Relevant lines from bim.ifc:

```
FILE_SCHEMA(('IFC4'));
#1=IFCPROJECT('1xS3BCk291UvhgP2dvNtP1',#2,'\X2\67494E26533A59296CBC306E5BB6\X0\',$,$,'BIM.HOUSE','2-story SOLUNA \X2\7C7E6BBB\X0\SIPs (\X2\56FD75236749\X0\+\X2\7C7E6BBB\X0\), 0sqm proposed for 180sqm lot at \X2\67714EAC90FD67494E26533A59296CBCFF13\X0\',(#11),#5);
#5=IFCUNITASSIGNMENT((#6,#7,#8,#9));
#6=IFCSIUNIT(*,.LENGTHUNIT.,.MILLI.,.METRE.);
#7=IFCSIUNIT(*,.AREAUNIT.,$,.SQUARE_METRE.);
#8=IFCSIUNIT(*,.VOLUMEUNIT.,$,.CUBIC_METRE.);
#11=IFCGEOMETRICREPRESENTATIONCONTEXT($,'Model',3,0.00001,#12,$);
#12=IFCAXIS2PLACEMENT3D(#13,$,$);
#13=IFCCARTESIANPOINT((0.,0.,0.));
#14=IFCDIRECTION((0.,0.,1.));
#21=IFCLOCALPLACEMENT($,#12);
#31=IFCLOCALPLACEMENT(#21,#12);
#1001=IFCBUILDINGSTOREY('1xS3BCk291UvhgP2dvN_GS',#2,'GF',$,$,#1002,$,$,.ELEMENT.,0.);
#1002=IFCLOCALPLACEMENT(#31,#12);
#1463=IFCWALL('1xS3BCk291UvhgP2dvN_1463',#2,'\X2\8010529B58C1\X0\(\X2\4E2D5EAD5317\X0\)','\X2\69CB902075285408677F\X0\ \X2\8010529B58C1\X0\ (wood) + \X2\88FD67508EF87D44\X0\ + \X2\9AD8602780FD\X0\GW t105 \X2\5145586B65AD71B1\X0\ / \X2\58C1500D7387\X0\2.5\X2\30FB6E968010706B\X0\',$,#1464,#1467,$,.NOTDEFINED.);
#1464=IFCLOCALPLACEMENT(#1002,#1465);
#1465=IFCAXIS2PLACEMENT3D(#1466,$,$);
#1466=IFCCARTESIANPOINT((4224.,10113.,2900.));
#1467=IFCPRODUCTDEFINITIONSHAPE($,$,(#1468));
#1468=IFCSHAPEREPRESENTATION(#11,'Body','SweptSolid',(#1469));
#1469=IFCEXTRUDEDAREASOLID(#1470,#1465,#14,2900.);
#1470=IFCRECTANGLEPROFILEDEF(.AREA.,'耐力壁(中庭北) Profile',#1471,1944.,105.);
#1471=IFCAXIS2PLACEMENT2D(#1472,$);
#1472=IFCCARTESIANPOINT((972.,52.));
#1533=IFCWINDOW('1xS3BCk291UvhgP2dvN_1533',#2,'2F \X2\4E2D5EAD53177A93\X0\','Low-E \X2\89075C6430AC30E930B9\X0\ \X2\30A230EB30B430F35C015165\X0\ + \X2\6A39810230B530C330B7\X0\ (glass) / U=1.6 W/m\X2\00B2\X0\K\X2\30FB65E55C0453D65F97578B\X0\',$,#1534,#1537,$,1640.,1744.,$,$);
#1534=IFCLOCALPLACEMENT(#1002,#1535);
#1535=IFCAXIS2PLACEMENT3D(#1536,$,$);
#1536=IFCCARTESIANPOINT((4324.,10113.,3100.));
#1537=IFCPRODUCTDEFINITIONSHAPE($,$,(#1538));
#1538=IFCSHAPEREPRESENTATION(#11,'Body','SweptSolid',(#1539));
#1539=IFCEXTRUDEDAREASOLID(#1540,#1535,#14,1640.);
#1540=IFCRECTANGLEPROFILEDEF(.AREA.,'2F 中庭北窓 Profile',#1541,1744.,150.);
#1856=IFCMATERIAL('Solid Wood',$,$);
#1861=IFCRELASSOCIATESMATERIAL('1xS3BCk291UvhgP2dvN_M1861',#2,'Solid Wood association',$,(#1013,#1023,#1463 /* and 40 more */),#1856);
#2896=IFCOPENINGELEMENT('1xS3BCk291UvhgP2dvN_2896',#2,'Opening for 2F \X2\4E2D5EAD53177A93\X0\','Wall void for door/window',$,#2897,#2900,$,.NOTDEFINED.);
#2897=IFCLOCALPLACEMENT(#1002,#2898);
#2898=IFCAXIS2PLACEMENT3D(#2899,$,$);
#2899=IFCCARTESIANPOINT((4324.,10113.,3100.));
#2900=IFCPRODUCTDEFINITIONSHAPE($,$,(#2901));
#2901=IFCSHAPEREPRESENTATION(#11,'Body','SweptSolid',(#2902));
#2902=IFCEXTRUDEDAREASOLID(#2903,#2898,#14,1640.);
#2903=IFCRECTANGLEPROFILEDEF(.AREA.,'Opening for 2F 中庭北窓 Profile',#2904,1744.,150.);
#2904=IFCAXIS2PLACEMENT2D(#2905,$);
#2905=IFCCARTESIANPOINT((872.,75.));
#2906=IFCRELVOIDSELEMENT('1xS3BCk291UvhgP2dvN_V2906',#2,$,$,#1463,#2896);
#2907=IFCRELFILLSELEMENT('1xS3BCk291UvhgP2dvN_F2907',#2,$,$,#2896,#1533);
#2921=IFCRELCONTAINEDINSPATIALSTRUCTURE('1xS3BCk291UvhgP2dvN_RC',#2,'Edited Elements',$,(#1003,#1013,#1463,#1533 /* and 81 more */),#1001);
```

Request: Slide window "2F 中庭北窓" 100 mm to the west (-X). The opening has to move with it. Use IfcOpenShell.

```python
import ifcopenshell
import ifcopenshell.api.geometry
import ifcopenshell.util.placement

model = ifcopenshell.open("bim.ifc")

window = model.by_guid("1xS3BCk291UvhgP2dvN_1533")
opening = window.FillsVoids[0].RelatingOpeningElement
wall = opening.VoidsElements[0].RelatingBuildingElement

wall_matrix = ifcopenshell.util.placement.get_local_placement(wall.ObjectPlacement)
shift = wall_matrix[:3, 0] * -100.0
before = ifcopenshell.util.placement.get_local_placement(window.ObjectPlacement)[:3, 3].copy()

# The window is not placed relative to its opening, so move both.
for product in (opening, window):
    matrix = ifcopenshell.util.placement.get_local_placement(product.ObjectPlacement)
    matrix[:3, 3] += shift
    ifcopenshell.api.geometry.edit_object_placement(model, product=product, matrix=matrix, is_si=False)

after = ifcopenshell.util.placement.get_local_placement(window.ObjectPlacement)[:3, 3]
print("window moved by", (after - before).round(3) + 0.0)

model.write("bim-out.ifc")
```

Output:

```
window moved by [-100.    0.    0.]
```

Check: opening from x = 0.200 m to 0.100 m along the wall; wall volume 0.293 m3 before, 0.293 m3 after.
